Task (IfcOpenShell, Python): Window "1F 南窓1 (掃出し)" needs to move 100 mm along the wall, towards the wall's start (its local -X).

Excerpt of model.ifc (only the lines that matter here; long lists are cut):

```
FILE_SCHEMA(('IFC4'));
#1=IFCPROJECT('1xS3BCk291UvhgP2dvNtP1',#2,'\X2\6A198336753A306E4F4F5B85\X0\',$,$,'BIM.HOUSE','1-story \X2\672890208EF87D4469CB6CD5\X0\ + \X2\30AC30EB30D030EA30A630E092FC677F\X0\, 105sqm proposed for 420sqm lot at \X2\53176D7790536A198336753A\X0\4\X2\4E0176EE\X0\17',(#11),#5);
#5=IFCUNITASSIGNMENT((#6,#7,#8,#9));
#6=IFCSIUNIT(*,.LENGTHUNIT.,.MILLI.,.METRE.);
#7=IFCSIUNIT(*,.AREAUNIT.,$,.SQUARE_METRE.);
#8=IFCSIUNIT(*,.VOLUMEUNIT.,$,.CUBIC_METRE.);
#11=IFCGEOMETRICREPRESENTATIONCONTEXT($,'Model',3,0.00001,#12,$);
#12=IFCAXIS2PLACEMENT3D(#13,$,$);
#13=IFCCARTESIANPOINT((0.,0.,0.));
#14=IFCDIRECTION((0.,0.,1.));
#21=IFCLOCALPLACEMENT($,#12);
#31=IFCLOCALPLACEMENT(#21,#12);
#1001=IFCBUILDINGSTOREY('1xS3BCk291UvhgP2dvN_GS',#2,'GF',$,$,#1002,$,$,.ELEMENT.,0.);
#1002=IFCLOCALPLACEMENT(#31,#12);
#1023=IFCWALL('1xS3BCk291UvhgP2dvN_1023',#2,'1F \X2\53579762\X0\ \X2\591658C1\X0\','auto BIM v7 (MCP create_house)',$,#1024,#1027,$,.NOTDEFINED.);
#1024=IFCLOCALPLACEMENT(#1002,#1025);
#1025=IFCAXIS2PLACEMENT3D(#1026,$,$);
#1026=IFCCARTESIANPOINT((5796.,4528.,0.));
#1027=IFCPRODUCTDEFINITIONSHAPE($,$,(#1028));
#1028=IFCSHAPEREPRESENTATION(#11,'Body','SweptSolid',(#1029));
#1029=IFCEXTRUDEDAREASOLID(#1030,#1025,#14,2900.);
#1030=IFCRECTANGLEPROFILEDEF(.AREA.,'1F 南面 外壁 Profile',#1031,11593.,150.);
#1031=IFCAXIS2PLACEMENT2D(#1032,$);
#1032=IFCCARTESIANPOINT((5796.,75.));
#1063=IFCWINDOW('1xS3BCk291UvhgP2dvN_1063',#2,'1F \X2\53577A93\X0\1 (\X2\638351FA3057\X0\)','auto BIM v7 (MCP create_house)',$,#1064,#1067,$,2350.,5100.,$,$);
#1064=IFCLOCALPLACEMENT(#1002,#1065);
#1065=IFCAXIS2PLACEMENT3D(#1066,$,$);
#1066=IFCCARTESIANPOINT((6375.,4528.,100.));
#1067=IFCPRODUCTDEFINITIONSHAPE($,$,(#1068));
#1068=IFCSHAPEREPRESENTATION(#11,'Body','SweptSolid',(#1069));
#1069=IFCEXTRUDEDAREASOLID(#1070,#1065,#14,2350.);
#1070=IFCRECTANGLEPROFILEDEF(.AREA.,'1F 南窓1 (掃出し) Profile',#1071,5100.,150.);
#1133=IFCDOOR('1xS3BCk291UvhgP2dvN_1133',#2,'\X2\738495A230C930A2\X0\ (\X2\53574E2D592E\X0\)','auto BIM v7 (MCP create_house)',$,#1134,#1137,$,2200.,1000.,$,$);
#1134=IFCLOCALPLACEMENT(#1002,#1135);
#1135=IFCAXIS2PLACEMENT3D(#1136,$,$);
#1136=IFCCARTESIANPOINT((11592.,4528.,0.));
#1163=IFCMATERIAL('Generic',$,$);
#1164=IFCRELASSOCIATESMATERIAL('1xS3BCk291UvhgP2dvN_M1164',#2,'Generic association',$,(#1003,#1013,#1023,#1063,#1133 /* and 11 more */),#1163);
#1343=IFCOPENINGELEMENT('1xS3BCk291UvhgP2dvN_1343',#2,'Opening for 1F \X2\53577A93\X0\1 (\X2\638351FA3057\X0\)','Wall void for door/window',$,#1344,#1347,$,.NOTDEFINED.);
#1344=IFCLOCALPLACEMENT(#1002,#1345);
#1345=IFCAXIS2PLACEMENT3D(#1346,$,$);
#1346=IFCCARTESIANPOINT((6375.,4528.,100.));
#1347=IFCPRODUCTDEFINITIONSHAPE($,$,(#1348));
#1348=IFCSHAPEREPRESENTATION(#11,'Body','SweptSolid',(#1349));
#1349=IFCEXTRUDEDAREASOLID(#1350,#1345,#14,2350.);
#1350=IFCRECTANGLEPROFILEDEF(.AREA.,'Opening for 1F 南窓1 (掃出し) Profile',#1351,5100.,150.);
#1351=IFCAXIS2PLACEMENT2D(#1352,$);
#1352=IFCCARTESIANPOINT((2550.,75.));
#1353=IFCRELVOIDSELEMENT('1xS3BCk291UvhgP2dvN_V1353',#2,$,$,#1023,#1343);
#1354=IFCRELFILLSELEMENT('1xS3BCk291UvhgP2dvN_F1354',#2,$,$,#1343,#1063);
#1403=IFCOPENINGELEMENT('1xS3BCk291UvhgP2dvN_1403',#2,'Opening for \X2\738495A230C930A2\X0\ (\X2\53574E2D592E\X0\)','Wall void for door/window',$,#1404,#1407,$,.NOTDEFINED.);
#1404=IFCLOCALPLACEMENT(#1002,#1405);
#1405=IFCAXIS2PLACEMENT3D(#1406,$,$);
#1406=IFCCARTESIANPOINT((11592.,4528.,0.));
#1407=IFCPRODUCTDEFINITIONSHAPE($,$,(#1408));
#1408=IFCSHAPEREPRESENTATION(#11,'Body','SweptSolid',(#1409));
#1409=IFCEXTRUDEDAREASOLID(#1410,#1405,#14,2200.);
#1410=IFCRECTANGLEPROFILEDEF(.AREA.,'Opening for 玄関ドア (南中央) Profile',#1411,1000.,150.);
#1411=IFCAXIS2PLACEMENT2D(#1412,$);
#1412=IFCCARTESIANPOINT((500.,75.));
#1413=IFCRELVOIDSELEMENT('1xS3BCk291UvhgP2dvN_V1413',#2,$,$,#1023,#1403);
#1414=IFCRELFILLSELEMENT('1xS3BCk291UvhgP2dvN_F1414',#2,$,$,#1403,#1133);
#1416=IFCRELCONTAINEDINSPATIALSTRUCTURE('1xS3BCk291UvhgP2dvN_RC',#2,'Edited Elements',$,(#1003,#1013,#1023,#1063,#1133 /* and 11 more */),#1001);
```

```python
import ifcopenshell
import ifcopenshell.api.geometry
import ifcopenshell.util.placement
import ifcopenshell.util.unit

model = ifcopenshell.open("model.ifc")
unit_scale = ifcopenshell.util.unit.calculate_unit_scale(model)

window = model.by_id(1063)
opening = window.FillsVoids[0].RelatingOpeningElement
wall = opening.VoidsElements[0].RelatingBuildingElement

wall_matrix = ifcopenshell.util.placement.get_local_placement(wall.ObjectPlacement)
shift = wall_matrix[:3, 0] * -0.1 / unit_scale
before = ifcopenshell.util.placement.get_local_placement(window.ObjectPlacement)[:3, 3].copy()

# The window is not placed relative to its opening, so move both.
for product in (opening, window):
    matrix = ifcopenshell.util.placement.get_local_placement(product.ObjectPlacement)
    matrix[:3, 3] += shift
    ifcopenshell.api.geometry.edit_object_placement(model, product=product, matrix=matrix, is_si=False)

after = ifcopenshell.util.placement.get_local_placement(window.ObjectPlacement)[:3, 3]
print("window moved by", (after - before).round(3) + 0.0)

model.write("model-out.ifc")
```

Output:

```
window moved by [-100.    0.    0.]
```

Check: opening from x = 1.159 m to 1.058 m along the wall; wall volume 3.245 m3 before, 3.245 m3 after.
